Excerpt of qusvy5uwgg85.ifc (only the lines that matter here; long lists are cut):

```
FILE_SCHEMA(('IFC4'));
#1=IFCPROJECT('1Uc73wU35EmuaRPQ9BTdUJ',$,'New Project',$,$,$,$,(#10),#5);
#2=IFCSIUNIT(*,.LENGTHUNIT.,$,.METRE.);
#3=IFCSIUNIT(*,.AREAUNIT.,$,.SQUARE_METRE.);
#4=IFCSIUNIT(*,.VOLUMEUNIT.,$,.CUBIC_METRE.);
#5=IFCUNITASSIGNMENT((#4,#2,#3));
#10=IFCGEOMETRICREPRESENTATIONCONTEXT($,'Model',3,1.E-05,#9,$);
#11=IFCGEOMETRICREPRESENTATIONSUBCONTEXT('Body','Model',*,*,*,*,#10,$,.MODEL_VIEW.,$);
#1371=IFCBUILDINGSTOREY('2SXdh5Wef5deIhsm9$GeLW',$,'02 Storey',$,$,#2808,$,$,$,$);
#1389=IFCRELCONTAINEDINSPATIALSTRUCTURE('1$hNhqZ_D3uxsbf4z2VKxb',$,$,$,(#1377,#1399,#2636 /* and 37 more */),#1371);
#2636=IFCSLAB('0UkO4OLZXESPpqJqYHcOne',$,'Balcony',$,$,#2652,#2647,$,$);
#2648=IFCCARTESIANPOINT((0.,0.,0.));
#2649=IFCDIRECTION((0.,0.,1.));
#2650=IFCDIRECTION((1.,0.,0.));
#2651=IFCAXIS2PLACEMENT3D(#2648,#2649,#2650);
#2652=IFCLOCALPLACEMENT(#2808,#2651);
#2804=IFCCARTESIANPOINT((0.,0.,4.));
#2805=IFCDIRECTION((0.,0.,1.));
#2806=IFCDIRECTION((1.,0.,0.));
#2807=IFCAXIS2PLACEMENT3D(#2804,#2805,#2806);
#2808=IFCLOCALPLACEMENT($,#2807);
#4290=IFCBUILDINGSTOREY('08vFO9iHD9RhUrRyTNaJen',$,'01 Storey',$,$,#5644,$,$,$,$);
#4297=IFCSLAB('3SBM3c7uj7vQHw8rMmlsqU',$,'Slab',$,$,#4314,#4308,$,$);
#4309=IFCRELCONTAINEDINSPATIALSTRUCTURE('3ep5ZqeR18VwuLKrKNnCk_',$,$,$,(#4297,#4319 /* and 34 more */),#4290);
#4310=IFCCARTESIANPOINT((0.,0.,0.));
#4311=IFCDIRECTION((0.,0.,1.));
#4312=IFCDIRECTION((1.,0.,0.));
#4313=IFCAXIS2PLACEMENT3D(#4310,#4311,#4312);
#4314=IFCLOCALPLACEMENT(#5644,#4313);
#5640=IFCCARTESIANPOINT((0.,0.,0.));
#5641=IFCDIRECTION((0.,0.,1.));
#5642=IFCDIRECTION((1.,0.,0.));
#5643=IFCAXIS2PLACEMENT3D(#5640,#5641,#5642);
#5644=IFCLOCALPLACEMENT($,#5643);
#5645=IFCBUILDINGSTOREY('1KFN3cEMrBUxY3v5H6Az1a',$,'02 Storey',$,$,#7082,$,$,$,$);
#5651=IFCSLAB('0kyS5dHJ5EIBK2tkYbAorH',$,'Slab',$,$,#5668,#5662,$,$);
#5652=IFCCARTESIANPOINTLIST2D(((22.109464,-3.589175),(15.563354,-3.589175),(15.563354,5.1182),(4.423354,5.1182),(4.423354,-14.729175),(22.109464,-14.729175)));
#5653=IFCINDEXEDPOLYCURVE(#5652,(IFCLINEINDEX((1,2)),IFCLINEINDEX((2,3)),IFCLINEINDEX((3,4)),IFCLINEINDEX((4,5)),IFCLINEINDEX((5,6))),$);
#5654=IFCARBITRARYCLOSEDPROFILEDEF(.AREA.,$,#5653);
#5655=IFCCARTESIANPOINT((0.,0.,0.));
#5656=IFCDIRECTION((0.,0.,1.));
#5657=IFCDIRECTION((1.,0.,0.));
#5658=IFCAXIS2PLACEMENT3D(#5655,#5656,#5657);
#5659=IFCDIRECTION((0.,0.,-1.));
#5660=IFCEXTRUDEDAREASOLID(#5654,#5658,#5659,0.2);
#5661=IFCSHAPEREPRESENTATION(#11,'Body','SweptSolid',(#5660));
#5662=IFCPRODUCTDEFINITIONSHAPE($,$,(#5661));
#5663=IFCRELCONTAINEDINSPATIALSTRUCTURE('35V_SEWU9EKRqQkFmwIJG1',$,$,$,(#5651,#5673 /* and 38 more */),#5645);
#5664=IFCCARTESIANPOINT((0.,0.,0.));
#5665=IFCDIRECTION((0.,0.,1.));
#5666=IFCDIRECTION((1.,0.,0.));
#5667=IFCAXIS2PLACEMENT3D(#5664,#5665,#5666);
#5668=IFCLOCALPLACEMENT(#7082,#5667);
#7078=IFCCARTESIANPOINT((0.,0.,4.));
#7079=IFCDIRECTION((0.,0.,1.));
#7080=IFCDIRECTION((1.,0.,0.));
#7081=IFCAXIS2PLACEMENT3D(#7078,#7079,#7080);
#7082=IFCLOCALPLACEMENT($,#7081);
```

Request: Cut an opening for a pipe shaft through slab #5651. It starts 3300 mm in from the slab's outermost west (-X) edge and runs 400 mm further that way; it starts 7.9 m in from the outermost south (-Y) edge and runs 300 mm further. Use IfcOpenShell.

```python
import numpy as np
import ifcopenshell
import ifcopenshell.api.feature
import ifcopenshell.api.geometry
import ifcopenshell.api.root
import ifcopenshell.geom
import ifcopenshell.util.placement
import ifcopenshell.util.representation
import ifcopenshell.util.shape
import ifcopenshell.util.unit

model = ifcopenshell.open("qusvy5uwgg85.ifc")
unit_scale = ifcopenshell.util.unit.calculate_unit_scale(model)
settings = ifcopenshell.geom.settings()


def volume(element):
    """Net volume in cubic metres, openings subtracted."""
    shape = ifcopenshell.geom.create_shape(settings, element)
    return ifcopenshell.util.shape.get_volume(shape.geometry)


slab = model.by_guid("0kyS5dHJ5EIBK2tkYbAorH")
before = volume(slab)

# Extent in the slab's own axes, in metres. The edges named are its -X and -Y sides.
slab_shape = ifcopenshell.geom.create_shape(settings, slab)
vertices = ifcopenshell.util.shape.get_vertices(slab_shape.geometry)
x_min, y_min, bottom = vertices.min(axis=0)
top = vertices[:, 2].max()

opening = ifcopenshell.api.root.create_entity(model, ifc_class="IfcOpeningElement", name="Pipe shaft opening", predefined_type="OPENING")
context = ifcopenshell.util.representation.get_context(model, "Model", "Body", "MODEL_VIEW")
width, depth = 0.4, 0.3
outline = [(0.0, 0.0), (width, 0.0), (width, depth), (0.0, depth), (0.0, 0.0)]
# Overshoot both faces by 50 mm so the cut is clean.
shape = ifcopenshell.api.geometry.add_slab_representation(
    model, context=context, depth=top - bottom + 0.1, polyline=outline
)
ifcopenshell.api.geometry.assign_representation(model, product=opening, representation=shape)

matrix = ifcopenshell.util.placement.get_local_placement(slab.ObjectPlacement)
matrix[:, 3] = matrix @ np.append(np.array([x_min + 3.3, y_min + 7.9, bottom - 0.05]) / unit_scale, 1.0)
ifcopenshell.api.geometry.edit_object_placement(model, product=opening, matrix=matrix, is_si=False)
ifcopenshell.api.feature.add_feature(model, feature=opening, element=slab)

after = volume(slab)

print(f"slab volume {before:.3f} -> {after:.3f} m3")

model.write("qusvy5uwgg85-out.ifc")
```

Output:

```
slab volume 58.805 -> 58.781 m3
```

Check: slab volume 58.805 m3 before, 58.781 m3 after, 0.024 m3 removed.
